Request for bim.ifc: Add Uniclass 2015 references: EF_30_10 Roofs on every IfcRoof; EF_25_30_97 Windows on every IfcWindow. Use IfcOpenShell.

First a look at what the model holds.

```python
import ifcopenshell

model = ifcopenshell.open("bim.ifc")
print(model.schema)
print("classifications:", [c.Name for c in model.by_type("IfcClassification")])
for ifc_class in ("IfcDoor", "IfcRoof", "IfcStair", "IfcWall", "IfcWindow"):
    print(ifc_class, len(model.by_type(ifc_class)))
```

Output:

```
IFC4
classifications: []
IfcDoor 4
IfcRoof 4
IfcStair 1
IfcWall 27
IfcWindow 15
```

```python
import ifcopenshell
import ifcopenshell.api.classification

model = ifcopenshell.open("bim.ifc")

system = ifcopenshell.api.classification.add_classification(model, classification="Uniclass 2015")

codes = {
    "IfcRoof": ("EF_30_10", "Roofs"),
    "IfcWindow": ("EF_25_30_97", "Windows"),
}
for ifc_class, (code, name) in codes.items():
    products = model.by_type(ifc_class)
    ifcopenshell.api.classification.add_reference(
        model, products=products, classification=system, identification=code, name=name
    )
    print(code, len(products))

model.write("bim_edited.ifc")
```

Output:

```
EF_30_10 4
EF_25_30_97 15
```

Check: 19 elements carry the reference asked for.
